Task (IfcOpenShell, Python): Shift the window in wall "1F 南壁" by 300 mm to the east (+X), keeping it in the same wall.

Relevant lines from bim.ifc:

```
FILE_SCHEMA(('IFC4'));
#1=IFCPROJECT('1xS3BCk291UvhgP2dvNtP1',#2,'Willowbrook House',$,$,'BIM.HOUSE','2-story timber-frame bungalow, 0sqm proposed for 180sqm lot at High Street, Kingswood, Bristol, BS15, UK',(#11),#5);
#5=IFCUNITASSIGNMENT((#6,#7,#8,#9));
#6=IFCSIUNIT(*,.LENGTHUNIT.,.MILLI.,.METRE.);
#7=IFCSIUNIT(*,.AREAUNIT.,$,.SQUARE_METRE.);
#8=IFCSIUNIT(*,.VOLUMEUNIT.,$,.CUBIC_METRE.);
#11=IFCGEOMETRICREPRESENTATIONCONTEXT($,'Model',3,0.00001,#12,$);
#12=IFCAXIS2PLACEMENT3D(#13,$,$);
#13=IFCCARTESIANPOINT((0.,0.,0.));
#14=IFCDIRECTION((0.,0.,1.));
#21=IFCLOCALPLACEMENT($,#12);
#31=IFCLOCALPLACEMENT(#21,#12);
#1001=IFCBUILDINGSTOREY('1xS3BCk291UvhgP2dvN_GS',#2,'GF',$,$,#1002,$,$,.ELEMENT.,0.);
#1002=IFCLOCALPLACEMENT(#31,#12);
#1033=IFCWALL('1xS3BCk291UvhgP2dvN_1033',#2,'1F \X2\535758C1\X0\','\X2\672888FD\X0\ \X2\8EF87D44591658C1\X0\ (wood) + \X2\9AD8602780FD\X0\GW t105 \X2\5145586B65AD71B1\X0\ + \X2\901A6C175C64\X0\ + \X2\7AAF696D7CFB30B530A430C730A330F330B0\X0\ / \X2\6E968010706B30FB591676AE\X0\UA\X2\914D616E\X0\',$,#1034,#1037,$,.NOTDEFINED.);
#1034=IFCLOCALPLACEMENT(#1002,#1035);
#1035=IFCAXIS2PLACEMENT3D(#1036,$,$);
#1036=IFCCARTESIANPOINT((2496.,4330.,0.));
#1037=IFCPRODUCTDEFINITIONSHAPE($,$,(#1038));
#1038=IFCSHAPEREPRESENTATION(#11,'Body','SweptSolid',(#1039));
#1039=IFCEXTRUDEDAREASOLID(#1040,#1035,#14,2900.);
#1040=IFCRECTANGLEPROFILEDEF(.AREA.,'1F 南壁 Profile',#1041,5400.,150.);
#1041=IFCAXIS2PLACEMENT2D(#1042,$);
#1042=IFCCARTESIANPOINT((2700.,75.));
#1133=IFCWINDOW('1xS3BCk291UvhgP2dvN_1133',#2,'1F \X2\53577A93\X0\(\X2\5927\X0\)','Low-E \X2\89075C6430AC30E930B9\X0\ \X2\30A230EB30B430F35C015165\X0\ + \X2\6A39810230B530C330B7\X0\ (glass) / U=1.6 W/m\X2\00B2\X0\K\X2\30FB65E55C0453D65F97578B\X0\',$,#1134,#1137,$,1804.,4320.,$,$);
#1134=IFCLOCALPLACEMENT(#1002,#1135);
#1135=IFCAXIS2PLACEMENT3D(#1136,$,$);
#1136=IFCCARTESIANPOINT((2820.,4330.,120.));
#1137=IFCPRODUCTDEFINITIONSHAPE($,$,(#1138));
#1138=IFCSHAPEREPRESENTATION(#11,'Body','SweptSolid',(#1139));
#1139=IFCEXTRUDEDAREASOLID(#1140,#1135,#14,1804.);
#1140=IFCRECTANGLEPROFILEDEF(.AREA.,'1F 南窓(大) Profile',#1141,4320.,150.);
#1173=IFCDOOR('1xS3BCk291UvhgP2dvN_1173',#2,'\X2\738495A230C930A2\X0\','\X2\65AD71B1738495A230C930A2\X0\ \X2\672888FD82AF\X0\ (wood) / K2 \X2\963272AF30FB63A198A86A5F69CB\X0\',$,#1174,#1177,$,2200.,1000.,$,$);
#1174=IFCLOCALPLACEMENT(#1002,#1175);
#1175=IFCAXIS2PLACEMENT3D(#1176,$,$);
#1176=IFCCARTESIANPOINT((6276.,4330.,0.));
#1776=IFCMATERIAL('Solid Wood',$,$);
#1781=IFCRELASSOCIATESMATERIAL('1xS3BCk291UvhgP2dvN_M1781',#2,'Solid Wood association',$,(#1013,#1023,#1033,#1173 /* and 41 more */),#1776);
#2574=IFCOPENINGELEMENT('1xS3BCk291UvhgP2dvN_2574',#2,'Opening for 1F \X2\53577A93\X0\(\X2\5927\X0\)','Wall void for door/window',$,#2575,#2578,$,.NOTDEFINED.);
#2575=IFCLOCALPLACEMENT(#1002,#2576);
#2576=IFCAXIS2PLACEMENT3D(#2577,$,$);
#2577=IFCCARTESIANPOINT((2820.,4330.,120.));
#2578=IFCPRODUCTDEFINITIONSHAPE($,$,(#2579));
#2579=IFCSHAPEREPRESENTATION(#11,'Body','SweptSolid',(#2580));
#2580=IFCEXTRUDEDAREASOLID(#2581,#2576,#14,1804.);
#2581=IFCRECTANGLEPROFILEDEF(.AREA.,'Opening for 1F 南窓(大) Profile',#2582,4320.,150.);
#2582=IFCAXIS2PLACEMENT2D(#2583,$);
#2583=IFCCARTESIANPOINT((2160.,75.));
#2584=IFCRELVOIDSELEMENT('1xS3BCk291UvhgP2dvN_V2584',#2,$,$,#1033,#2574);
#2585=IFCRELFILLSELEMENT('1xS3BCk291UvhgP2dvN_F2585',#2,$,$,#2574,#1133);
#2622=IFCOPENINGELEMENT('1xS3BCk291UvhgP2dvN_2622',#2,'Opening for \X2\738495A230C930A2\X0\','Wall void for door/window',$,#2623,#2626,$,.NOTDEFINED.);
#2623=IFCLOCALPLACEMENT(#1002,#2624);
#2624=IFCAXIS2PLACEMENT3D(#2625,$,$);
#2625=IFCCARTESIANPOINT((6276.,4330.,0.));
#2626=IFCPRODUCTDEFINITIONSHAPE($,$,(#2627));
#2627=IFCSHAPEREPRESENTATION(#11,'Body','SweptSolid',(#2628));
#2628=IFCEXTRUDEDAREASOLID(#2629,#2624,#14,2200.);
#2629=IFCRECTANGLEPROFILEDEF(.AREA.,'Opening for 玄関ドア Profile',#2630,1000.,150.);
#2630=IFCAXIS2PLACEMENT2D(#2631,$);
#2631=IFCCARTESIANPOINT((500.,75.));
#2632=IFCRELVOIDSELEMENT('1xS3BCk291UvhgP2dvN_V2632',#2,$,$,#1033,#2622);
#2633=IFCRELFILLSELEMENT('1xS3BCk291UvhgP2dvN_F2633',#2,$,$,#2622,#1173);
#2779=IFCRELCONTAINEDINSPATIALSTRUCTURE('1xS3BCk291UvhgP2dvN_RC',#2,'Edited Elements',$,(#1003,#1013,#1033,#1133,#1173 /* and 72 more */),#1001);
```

```python
import ifcopenshell
import ifcopenshell.api.geometry
import ifcopenshell.util.placement
import ifcopenshell.util.unit

model = ifcopenshell.open("bim.ifc")
unit_scale = ifcopenshell.util.unit.calculate_unit_scale(model)

window = model.by_guid("1xS3BCk291UvhgP2dvN_1133")
opening = window.FillsVoids[0].RelatingOpeningElement
wall = opening.VoidsElements[0].RelatingBuildingElement

wall_matrix = ifcopenshell.util.placement.get_local_placement(wall.ObjectPlacement)
shift = wall_matrix[:3, 0] * 0.3 / unit_scale
before = ifcopenshell.util.placement.get_local_placement(window.ObjectPlacement)[:3, 3].copy()

# The window is not placed relative to its opening, so move both.
for product in (opening, window):
    matrix = ifcopenshell.util.placement.get_local_placement(product.ObjectPlacement)
    matrix[:3, 3] += shift
    ifcopenshell.api.geometry.edit_object_placement(model, product=product, matrix=matrix, is_si=False)

after = ifcopenshell.util.placement.get_local_placement(window.ObjectPlacement)[:3, 3]
print("window moved by", (after - before).round(3) + 0.0)

model.write("bim_edited.ifc")
```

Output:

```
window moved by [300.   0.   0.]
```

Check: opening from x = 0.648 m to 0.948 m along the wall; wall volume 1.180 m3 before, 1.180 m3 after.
